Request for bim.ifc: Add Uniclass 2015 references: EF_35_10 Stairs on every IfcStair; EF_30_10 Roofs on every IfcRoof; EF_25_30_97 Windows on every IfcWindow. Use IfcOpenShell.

First a look at what the model holds.

```python
import ifcopenshell

model = ifcopenshell.open("bim.ifc")
print(model.schema)
print("classifications:", [c.Name for c in model.by_type("IfcClassification")])
for ifc_class in ("IfcDoor", "IfcRoof", "IfcStair", "IfcWall", "IfcWindow"):
    print(ifc_class, len(model.by_type(ifc_class)))
```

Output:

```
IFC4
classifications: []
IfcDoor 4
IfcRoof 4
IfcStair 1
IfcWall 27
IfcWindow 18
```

```python
import ifcopenshell
import ifcopenshell.api.classification

model = ifcopenshell.open("bim.ifc")

system = ifcopenshell.api.classification.add_classification(model, classification="Uniclass 2015")

codes = {
    "IfcStair": ("EF_35_10", "Stairs"),
    "IfcRoof": ("EF_30_10", "Roofs"),
    "IfcWindow": ("EF_25_30_97", "Windows"),
}
for ifc_class, (code, name) in codes.items():
    products = model.by_type(ifc_class)
    ifcopenshell.api.classification.add_reference(
        model, products=products, classification=system, identification=code, name=name
    )
    print(code, len(products))

model.write("bim_edited.ifc")
```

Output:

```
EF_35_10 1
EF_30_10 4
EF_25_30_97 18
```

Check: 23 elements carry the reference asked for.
